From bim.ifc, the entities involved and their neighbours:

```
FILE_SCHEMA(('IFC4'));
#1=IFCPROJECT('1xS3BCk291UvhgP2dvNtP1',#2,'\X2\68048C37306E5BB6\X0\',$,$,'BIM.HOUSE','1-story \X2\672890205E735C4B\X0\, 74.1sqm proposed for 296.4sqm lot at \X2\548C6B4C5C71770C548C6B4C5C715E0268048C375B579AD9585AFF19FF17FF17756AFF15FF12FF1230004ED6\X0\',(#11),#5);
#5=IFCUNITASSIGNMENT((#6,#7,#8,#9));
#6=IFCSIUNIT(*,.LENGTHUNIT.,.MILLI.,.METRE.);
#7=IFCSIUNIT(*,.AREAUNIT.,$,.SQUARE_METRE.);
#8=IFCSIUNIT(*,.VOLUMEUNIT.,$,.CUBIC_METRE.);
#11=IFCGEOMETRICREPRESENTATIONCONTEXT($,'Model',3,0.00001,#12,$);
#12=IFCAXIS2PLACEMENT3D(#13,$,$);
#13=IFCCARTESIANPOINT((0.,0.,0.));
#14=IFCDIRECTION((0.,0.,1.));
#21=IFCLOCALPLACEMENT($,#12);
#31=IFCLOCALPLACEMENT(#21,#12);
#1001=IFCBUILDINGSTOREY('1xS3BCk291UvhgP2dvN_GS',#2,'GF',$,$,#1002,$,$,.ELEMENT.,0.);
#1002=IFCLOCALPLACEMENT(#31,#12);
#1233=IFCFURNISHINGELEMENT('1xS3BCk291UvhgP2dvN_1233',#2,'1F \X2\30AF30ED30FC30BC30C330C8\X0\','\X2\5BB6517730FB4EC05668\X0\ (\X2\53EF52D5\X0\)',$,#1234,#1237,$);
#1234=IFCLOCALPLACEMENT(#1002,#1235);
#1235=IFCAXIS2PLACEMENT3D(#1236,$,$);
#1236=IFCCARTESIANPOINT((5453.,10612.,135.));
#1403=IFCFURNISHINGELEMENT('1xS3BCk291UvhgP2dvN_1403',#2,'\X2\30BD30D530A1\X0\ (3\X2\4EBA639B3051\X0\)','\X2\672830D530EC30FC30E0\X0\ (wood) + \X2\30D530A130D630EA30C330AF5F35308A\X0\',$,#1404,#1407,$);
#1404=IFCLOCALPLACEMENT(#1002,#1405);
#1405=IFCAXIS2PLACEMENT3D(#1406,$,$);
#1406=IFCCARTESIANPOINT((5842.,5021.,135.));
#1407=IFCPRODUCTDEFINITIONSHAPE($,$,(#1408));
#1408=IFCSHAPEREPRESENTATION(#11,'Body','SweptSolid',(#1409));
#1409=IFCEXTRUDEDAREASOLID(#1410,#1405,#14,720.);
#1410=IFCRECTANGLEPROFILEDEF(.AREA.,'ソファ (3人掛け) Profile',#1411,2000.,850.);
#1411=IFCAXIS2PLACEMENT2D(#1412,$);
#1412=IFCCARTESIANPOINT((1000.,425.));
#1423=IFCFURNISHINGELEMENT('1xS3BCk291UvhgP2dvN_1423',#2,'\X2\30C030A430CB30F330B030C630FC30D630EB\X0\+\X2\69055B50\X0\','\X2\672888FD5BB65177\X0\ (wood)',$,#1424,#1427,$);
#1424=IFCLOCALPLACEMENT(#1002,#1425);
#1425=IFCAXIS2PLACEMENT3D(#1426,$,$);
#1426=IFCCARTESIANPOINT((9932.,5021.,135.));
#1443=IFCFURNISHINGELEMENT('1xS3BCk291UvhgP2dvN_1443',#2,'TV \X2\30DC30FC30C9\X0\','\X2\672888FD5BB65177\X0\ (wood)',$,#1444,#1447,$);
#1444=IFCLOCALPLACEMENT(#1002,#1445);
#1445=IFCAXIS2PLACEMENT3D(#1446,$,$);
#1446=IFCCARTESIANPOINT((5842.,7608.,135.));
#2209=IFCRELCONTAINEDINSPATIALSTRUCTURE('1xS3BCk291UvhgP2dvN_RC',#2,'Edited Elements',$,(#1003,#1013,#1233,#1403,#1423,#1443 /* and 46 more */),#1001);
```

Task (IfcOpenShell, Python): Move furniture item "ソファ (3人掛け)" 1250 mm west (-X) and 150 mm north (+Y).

```python
import ifcopenshell
import ifcopenshell.api.geometry
import ifcopenshell.util.placement
import ifcopenshell.util.unit

model = ifcopenshell.open("bim.ifc")
unit_scale = ifcopenshell.util.unit.calculate_unit_scale(model)

item = model.by_id(1403)
matrix = ifcopenshell.util.placement.get_local_placement(item.ObjectPlacement)
matrix[0, 3] -= 1.25 / unit_scale
matrix[1, 3] += 0.15 / unit_scale
ifcopenshell.api.geometry.edit_object_placement(model, product=item, matrix=matrix, is_si=False)

print(ifcopenshell.util.placement.get_local_placement(item.ObjectPlacement).round(3) + 0.0)

model.write("bim_edited.ifc")
```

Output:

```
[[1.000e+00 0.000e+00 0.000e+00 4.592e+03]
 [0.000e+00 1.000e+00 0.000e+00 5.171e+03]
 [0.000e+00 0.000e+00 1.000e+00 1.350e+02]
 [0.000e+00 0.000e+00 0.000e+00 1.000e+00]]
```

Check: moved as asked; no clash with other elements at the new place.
